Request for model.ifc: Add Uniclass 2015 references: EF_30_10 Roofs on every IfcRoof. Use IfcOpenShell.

First a look at what the model holds.

```python
import ifcopenshell

model = ifcopenshell.open("model.ifc")
print(model.schema)
print("classifications:", [c.Name for c in model.by_type("IfcClassification")])
for ifc_class in ("IfcDoor", "IfcRoof", "IfcStair", "IfcWall", "IfcWindow"):
    print(ifc_class, len(model.by_type(ifc_class)))
```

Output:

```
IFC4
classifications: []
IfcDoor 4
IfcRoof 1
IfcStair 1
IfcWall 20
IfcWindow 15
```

```python
import ifcopenshell
import ifcopenshell.api.classification

model = ifcopenshell.open("model.ifc")

system = ifcopenshell.api.classification.add_classification(model, classification="Uniclass 2015")

codes = {
    "IfcRoof": ("EF_30_10", "Roofs"),
}
for ifc_class, (code, name) in codes.items():
    products = model.by_type(ifc_class)
    ifcopenshell.api.classification.add_reference(
        model, products=products, classification=system, identification=code, name=name
    )
    print(code, len(products))

model.write("model_v2.ifc")
```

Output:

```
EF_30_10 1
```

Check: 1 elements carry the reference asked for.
